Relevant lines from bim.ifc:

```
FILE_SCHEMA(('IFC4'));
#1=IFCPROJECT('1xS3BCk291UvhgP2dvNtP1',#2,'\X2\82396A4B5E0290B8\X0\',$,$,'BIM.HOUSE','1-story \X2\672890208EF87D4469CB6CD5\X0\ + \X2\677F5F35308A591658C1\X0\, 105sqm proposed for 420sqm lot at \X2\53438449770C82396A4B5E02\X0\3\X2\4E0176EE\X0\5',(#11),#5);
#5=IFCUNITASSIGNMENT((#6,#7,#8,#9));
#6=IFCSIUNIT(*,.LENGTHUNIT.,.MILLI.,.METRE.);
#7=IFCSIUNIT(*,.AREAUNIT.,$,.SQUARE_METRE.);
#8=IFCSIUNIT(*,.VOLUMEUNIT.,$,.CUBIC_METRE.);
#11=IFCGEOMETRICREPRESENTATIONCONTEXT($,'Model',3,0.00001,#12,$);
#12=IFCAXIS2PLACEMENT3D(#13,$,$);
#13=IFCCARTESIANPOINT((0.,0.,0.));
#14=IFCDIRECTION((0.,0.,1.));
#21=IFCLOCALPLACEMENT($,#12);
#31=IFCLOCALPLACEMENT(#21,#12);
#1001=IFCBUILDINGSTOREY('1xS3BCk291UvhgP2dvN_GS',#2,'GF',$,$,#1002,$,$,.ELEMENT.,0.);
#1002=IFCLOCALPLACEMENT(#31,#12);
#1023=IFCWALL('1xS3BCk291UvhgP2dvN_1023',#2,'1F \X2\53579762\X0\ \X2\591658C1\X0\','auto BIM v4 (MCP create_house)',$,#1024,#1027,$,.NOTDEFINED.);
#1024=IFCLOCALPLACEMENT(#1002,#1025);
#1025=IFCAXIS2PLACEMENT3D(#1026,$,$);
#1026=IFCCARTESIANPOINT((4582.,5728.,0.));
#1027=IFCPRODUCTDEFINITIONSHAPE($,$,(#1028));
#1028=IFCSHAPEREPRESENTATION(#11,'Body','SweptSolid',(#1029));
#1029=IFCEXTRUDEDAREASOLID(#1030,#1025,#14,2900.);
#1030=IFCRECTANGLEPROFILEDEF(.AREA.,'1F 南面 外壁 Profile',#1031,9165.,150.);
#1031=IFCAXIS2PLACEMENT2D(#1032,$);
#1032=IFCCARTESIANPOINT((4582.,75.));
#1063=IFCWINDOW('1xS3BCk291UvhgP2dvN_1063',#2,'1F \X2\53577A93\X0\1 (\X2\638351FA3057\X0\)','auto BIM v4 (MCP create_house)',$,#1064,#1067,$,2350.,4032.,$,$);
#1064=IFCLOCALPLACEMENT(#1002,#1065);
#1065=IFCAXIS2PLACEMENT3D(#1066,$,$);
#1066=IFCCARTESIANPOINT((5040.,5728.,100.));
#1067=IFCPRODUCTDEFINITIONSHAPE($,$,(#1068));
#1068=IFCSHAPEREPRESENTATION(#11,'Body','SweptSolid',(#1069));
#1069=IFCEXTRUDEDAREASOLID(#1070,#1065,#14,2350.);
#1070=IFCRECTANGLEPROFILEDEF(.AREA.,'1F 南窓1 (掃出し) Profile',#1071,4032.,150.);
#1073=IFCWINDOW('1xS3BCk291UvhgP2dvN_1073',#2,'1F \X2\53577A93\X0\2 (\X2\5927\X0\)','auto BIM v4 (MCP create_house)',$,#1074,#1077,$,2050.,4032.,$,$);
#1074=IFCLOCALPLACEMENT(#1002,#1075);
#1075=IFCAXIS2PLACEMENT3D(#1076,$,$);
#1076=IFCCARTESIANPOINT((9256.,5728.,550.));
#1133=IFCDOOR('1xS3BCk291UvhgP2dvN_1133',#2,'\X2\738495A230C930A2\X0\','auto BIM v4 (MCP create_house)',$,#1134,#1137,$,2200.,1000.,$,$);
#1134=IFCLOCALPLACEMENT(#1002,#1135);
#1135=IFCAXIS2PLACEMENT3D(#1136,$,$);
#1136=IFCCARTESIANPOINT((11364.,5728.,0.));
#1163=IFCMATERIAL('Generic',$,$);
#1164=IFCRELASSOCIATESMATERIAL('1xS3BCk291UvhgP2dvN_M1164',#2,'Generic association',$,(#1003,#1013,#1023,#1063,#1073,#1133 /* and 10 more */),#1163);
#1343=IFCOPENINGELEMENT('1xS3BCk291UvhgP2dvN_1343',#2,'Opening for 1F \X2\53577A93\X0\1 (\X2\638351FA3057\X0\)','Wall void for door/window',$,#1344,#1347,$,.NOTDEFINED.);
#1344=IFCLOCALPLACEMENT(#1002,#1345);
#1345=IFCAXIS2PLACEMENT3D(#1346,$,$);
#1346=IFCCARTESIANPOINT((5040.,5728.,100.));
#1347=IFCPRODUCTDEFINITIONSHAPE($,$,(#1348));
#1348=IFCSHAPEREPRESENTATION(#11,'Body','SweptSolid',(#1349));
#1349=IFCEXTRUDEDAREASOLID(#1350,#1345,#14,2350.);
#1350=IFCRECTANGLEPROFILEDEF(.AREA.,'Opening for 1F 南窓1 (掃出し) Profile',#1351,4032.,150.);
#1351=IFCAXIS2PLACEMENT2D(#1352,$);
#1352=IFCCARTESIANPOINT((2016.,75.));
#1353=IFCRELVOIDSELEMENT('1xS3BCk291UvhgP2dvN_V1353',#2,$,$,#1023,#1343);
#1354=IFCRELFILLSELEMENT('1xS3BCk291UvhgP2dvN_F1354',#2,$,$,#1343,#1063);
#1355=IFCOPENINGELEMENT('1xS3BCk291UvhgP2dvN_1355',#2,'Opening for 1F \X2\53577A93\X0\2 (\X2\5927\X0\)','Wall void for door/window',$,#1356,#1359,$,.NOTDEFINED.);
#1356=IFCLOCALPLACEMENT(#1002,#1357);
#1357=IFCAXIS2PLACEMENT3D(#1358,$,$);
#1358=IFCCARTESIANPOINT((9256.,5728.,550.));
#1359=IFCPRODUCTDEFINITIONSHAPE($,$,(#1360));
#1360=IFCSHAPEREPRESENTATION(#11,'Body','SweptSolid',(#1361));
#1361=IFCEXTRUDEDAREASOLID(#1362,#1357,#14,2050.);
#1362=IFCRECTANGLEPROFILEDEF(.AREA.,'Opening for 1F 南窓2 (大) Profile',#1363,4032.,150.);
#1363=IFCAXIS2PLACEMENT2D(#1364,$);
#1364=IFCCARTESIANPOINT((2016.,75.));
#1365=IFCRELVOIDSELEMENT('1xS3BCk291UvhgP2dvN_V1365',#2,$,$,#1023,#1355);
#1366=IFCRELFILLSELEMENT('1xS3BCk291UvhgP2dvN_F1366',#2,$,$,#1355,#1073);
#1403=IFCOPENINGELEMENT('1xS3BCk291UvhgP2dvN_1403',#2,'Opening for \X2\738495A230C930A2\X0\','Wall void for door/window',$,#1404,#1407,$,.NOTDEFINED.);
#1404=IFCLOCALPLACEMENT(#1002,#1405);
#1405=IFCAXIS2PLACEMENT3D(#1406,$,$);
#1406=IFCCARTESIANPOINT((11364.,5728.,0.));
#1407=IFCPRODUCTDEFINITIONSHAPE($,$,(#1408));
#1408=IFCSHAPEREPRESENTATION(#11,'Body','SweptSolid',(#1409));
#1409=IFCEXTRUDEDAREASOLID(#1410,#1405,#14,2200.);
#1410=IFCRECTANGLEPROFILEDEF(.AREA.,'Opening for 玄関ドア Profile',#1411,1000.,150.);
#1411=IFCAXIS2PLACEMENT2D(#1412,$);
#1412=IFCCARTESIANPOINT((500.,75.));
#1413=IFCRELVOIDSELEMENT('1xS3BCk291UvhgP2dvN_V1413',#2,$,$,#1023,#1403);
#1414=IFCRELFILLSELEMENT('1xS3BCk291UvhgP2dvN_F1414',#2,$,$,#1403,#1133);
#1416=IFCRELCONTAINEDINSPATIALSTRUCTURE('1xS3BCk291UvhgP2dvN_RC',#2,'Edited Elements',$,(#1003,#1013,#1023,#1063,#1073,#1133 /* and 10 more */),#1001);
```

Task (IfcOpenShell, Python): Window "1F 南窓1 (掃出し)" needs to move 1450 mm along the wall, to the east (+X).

```python
import ifcopenshell
import ifcopenshell.api.geometry
import ifcopenshell.util.placement
import ifcopenshell.util.unit

model = ifcopenshell.open("bim.ifc")
unit_scale = ifcopenshell.util.unit.calculate_unit_scale(model)

window = model.by_id(1063)
opening = window.FillsVoids[0].RelatingOpeningElement
wall = opening.VoidsElements[0].RelatingBuildingElement

wall_matrix = ifcopenshell.util.placement.get_local_placement(wall.ObjectPlacement)
shift = wall_matrix[:3, 0] * 1.45 / unit_scale
before = ifcopenshell.util.placement.get_local_placement(window.ObjectPlacement)[:3, 3].copy()

# The window is not placed relative to its opening, so move both.
for product in (opening, window):
    matrix = ifcopenshell.util.placement.get_local_placement(product.ObjectPlacement)
    matrix[:3, 3] += shift
    ifcopenshell.api.geometry.edit_object_placement(model, product=product, matrix=matrix, is_si=False)

after = ifcopenshell.util.placement.get_local_placement(window.ObjectPlacement)[:3, 3]
print("window moved by", (after - before).round(3) + 0.0)

model.write("bim_v2.ifc")
```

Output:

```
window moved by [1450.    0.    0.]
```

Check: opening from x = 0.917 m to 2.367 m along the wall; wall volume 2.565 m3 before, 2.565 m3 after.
